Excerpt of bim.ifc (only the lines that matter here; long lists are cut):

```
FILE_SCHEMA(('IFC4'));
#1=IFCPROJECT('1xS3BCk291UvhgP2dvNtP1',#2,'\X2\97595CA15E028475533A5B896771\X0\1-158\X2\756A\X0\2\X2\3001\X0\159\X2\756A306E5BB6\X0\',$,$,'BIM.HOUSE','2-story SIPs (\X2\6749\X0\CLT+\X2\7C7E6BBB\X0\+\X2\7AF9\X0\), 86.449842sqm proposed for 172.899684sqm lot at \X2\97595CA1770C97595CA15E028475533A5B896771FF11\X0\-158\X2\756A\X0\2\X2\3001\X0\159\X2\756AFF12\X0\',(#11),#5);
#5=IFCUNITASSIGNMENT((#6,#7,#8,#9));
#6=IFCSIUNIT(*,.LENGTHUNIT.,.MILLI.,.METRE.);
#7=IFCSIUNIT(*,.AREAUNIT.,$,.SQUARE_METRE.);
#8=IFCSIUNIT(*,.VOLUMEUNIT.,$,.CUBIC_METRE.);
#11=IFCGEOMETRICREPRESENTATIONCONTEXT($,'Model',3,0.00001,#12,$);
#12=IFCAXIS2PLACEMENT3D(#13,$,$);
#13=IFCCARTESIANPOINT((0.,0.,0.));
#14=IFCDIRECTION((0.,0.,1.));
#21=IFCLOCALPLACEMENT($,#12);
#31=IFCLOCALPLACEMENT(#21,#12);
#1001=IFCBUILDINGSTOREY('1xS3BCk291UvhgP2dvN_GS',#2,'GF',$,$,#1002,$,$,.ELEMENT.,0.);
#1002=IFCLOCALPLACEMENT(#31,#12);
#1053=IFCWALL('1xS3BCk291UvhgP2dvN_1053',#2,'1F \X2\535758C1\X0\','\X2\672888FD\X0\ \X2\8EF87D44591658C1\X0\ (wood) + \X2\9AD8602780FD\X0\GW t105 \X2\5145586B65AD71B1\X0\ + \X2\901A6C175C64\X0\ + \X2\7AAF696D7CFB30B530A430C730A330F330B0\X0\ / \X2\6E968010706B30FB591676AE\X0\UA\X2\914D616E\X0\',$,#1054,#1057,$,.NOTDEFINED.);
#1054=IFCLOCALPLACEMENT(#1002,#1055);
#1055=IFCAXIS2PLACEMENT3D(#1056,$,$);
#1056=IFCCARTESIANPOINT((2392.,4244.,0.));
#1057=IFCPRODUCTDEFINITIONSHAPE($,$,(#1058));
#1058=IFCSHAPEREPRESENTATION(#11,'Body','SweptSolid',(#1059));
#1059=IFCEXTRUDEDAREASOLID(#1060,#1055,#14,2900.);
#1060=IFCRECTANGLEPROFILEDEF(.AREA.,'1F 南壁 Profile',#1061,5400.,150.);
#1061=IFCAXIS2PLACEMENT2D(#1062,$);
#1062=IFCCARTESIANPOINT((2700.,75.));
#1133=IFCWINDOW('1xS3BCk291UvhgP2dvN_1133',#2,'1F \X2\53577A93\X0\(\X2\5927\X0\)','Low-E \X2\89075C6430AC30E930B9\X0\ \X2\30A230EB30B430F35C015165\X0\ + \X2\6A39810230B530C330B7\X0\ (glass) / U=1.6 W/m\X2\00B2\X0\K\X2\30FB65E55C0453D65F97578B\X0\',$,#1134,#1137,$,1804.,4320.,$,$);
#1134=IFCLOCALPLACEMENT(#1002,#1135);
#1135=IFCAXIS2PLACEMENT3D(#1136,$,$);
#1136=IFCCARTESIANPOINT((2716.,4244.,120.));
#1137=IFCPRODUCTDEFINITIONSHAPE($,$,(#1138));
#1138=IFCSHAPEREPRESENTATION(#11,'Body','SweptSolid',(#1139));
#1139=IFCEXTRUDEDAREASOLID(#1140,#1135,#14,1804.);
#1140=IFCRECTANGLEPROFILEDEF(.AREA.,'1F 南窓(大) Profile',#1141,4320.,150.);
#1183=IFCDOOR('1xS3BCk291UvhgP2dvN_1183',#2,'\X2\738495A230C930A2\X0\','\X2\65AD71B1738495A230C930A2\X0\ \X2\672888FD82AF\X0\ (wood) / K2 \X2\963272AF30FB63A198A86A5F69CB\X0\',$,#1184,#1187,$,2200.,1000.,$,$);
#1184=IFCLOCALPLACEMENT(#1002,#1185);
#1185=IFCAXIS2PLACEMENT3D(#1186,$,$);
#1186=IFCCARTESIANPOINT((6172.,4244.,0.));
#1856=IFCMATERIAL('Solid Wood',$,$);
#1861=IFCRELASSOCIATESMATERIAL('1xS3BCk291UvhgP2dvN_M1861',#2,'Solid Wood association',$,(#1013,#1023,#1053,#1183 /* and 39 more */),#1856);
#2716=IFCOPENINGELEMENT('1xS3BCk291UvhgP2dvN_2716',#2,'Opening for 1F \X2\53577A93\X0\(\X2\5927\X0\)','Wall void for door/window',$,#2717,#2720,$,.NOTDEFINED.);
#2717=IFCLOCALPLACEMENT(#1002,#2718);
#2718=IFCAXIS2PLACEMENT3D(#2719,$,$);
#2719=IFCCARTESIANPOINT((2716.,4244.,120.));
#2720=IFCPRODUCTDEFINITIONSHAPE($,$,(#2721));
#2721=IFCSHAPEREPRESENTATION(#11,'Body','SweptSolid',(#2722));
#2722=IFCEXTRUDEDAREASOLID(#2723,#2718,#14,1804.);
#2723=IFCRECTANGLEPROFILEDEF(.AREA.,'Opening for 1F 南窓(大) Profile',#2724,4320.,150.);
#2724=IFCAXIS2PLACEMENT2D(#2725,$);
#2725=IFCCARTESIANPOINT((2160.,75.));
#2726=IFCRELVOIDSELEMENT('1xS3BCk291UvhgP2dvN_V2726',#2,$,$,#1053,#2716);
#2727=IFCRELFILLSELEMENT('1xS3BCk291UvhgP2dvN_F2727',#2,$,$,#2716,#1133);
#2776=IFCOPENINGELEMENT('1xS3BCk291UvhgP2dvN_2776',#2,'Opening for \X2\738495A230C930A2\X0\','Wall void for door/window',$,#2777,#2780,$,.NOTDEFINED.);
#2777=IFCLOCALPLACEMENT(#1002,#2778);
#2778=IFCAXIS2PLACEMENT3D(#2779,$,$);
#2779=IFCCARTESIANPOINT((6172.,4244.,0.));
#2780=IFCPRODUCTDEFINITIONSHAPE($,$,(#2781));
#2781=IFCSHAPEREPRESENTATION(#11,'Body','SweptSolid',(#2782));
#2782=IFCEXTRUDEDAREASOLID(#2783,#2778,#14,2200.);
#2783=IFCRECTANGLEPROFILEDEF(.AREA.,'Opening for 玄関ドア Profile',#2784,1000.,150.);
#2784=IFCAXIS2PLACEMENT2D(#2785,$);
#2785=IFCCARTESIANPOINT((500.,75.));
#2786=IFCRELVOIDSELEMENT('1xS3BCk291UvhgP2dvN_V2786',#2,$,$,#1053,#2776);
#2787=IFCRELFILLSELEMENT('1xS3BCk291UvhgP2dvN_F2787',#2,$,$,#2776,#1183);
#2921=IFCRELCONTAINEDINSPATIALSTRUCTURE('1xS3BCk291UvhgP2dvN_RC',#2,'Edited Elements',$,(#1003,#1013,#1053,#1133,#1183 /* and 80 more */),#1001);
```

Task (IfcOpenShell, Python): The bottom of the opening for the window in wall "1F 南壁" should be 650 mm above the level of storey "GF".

```python
import numpy as np
import ifcopenshell
import ifcopenshell.api.geometry
import ifcopenshell.geom
import ifcopenshell.util.element
import ifcopenshell.util.placement
import ifcopenshell.util.shape
import ifcopenshell.util.unit

model = ifcopenshell.open("bim.ifc")
unit_scale = ifcopenshell.util.unit.calculate_unit_scale(model)

window = model.by_guid("1xS3BCk291UvhgP2dvN_1133")
opening = window.FillsVoids[0].RelatingOpeningElement
storey = ifcopenshell.util.element.get_container(window, ifc_class="IfcBuildingStorey")
level = ifcopenshell.util.placement.get_local_placement(storey.ObjectPlacement)[2, 3]

# The opening's origin need not be at the sill, so measure its lowest point.
shape = ifcopenshell.geom.create_shape(ifcopenshell.geom.settings(), opening)
bottom = ifcopenshell.util.shape.get_shape_bottom_elevation(shape, shape.geometry) / unit_scale
dz = level + 650.0 - bottom

shift = np.array([0.0, 0.0, dz])
# The window is not placed relative to its opening, so move both.
for product in (opening, window):
    matrix = ifcopenshell.util.placement.get_local_placement(product.ObjectPlacement)
    matrix[:3, 3] += shift
    ifcopenshell.api.geometry.edit_object_placement(model, product=product, matrix=matrix, is_si=False)

print(f"moved by {dz * unit_scale:+.3f} m")

model.write("bim_edited.ifc")
```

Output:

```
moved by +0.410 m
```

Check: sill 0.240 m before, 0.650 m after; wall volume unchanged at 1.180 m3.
